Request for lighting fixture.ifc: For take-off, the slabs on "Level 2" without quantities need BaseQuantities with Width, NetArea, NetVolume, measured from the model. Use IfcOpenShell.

First a look at what the model holds.

```python
import ifcopenshell
import ifcopenshell.util.element
import ifcopenshell.util.unit

model = ifcopenshell.open("lighting fixture.ifc")
print(model.schema)
for unit_type in ("LENGTHUNIT", "AREAUNIT", "VOLUMEUNIT"):
    print(unit_type, ifcopenshell.util.unit.calculate_unit_scale(model, unit_type))
storey = next(s for s in model.by_type("IfcBuildingStorey") if s.Name == "Level 2")
slabs = [e for e in ifcopenshell.util.element.get_decomposition(storey) if e.is_a("IfcSlab")]
for e in sorted(slabs, key=lambda e: e.id()):
    print(e.id(), e.is_a(), e.Name, list(ifcopenshell.util.element.get_psets(e, qtos_only=True)), sep=" | ")
```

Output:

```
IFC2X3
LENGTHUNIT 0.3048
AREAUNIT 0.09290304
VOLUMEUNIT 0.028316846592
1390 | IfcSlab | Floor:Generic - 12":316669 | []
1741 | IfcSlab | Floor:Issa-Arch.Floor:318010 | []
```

```python
import ifcopenshell
import ifcopenshell.api.pset
import ifcopenshell.geom
import ifcopenshell.util.element
import ifcopenshell.util.shape
import ifcopenshell.util.unit

model = ifcopenshell.open("lighting fixture.ifc")
unit_scale = ifcopenshell.util.unit.calculate_unit_scale(model)
area_scale = ifcopenshell.util.unit.calculate_unit_scale(model, "AREAUNIT")
volume_scale = ifcopenshell.util.unit.calculate_unit_scale(model, "VOLUMEUNIT")
settings = ifcopenshell.geom.settings()

storey = next(s for s in model.by_type("IfcBuildingStorey") if s.Name == "Level 2")
slabs = [e for e in ifcopenshell.util.element.get_decomposition(storey) if e.is_a("IfcSlab")]

for e in sorted(slabs, key=lambda e: e.id()):
    if ifcopenshell.util.element.get_psets(e, qtos_only=True, should_inherit=False):
        continue
    # Geometry comes back in metres, in the element's own axes.
    shape = ifcopenshell.geom.create_shape(settings, e)
    values = {
        "Width": ifcopenshell.util.shape.get_z(shape.geometry) / unit_scale,
        "NetArea": ifcopenshell.util.shape.get_footprint_area(shape.geometry) / area_scale,
        "NetVolume": ifcopenshell.util.shape.get_volume(shape.geometry) / volume_scale,
    }
    qto = ifcopenshell.api.pset.add_qto(model, product=e, name="BaseQuantities")
    ifcopenshell.api.pset.edit_qto(model, qto=qto, properties=values)
    print(e.id(), {k: round(v, 3) for k, v in values.items()})

model.write("lighting fixture_updated.ifc")
```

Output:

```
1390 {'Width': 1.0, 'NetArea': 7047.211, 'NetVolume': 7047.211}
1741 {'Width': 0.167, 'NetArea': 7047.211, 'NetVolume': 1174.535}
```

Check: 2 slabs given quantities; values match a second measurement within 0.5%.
